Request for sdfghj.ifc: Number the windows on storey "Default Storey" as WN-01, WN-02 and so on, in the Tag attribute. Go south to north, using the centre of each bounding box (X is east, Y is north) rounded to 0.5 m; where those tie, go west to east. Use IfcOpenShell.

First a look at what the model holds.

```python
import ifcopenshell
import ifcopenshell.util.element
import ifcopenshell.util.placement

model = ifcopenshell.open("sdfghj.ifc")
print(model.schema)
storey = next(s for s in model.by_type("IfcBuildingStorey") if s.Name == "Default Storey")
windows = [e for e in ifcopenshell.util.element.get_decomposition(storey) if e.is_a("IfcWindow")]
for e in sorted(windows, key=lambda e: e.id()):
    origin = ifcopenshell.util.placement.get_local_placement(e.ObjectPlacement)[:3, 3]
    print(e.id(), e.Tag, e.Name, origin.round(2) + 0.0, sep=" | ")
```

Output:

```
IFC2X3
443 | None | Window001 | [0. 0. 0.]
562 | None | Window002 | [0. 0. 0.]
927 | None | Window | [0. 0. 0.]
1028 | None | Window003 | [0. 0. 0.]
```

```python
import ifcopenshell
import ifcopenshell.geom
import ifcopenshell.util.element
import ifcopenshell.util.shape

model = ifcopenshell.open("sdfghj.ifc")
settings = ifcopenshell.geom.settings()
settings.set("use-world-coords", True)


def centre(element):
    shape = ifcopenshell.geom.create_shape(settings, element)
    return ifcopenshell.util.shape.get_bbox_centroid(shape.geometry)


storey = next(s for s in model.by_type("IfcBuildingStorey") if s.Name == "Default Storey")
windows = [e for e in ifcopenshell.util.element.get_decomposition(storey) if e.is_a("IfcWindow")]

# Insertion points can sit at a corner or the storey origin, so sort by the geometry (in metres).
centres = {e: centre(e) for e in windows}
windows.sort(key=lambda e: (round(centres[e][1] / 0.5), centres[e][0]))

for i, e in enumerate(windows, start=1):
    number = f"WN-{i:02d}"
    e.Tag = number
    print(e.id(), number)

model.write("sdfghj_updated.ifc")
```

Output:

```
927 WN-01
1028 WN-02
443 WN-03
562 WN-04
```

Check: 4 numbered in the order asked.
